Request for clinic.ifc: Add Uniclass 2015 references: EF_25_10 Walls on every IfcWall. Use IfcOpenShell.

First a look at what the model holds.

```python
import ifcopenshell

model = ifcopenshell.open("clinic.ifc")
print(model.schema)
print("classifications:", [c.Name for c in model.by_type("IfcClassification")])
for ifc_class in ("IfcDoor", "IfcRoof", "IfcStair", "IfcWall", "IfcWindow"):
    print(ifc_class, len(model.by_type(ifc_class)))
```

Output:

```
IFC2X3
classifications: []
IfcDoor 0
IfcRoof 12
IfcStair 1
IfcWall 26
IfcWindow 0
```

```python
import ifcopenshell
import ifcopenshell.api.classification

model = ifcopenshell.open("clinic.ifc")

# IFC2X3 requires Source and Edition and has no link from the project to the system.
system = model.create_entity("IfcClassification", Source="NBS", Edition="2015", Name="Uniclass 2015")

codes = {
    "IfcWall": ("EF_25_10", "Walls"),
}
for ifc_class, (code, name) in codes.items():
    products = model.by_type(ifc_class)
    ifcopenshell.api.classification.add_reference(
        model, products=products, classification=system, identification=code, name=name
    )
    print(code, len(products))

model.write("clinic_updated.ifc")
```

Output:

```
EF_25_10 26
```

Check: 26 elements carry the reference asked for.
